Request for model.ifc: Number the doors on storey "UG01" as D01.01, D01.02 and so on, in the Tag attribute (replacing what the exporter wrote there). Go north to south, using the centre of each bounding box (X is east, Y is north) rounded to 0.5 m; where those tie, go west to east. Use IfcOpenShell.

First a look at what the model holds.

```python
import ifcopenshell
import ifcopenshell.util.element
import ifcopenshell.util.placement

model = ifcopenshell.open("model.ifc")
print(model.schema)
storey = next(s for s in model.by_type("IfcBuildingStorey") if s.Name == "UG01")
doors = [e for e in ifcopenshell.util.element.get_decomposition(storey) if e.is_a("IfcDoor")]
for e in sorted(doors, key=lambda e: e.id()):
    origin = ifcopenshell.util.placement.get_local_placement(e.ObjectPlacement)[:3, 3]
    print(e.id(), e.Tag, e.Name, origin.round(2) + 0.0, sep=" | ")
```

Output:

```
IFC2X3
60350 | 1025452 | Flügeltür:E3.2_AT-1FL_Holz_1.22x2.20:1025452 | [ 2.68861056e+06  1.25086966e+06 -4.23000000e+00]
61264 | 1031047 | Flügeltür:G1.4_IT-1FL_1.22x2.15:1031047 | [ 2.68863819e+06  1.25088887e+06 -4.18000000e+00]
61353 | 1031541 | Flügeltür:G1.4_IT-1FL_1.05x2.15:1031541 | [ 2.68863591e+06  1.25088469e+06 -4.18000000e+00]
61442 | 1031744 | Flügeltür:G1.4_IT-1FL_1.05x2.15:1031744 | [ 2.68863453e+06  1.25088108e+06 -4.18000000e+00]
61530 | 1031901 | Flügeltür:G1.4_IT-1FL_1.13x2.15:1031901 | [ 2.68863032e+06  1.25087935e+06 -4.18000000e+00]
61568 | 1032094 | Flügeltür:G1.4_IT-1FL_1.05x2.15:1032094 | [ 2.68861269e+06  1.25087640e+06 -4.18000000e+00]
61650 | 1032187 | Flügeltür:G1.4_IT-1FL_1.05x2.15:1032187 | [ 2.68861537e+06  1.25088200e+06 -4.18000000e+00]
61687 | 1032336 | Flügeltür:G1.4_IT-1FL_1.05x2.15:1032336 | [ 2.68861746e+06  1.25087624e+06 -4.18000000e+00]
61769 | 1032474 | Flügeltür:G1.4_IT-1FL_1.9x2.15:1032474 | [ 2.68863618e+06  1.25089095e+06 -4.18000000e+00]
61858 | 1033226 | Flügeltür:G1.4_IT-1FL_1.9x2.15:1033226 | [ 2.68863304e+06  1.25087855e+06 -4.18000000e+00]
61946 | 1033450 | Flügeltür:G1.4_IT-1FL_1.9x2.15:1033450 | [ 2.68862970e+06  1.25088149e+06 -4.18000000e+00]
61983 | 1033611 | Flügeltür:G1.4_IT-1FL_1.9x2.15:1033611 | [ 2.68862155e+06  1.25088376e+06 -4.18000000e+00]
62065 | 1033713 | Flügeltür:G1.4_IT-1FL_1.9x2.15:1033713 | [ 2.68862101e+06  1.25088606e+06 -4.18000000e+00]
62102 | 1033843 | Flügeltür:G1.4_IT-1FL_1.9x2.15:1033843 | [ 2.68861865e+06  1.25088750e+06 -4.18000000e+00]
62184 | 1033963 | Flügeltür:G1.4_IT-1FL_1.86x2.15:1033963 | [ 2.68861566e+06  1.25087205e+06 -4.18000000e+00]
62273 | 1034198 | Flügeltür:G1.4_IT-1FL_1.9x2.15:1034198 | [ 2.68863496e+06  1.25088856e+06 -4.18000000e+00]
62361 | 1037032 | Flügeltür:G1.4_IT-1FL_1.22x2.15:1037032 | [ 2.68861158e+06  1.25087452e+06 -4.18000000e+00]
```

```python
import ifcopenshell
import ifcopenshell.geom
import ifcopenshell.util.element
import ifcopenshell.util.shape

model = ifcopenshell.open("model.ifc")
settings = ifcopenshell.geom.settings()
settings.set("use-world-coords", True)


def centre(element):
    shape = ifcopenshell.geom.create_shape(settings, element)
    return ifcopenshell.util.shape.get_bbox_centroid(shape.geometry)


storey = next(s for s in model.by_type("IfcBuildingStorey") if s.Name == "UG01")
doors = [e for e in ifcopenshell.util.element.get_decomposition(storey) if e.is_a("IfcDoor")]

# Insertion points can sit at a corner or the storey origin, so sort by the geometry (in metres).
centres = {e: centre(e) for e in doors}
doors.sort(key=lambda e: (-round(centres[e][1] / 0.5), centres[e][0]))

for i, e in enumerate(doors, start=1):
    number = f"D01.{i:02d}"
    e.Tag = number
    print(e.id(), number)

model.write("model-out.ifc")
```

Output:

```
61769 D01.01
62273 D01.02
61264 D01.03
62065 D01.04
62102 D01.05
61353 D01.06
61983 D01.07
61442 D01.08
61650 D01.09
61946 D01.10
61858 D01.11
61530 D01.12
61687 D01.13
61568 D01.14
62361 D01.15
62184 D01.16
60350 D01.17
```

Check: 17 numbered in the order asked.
